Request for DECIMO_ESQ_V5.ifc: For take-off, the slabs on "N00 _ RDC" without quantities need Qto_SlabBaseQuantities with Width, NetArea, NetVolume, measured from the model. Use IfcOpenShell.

First a look at what the model holds.

```python
import ifcopenshell
import ifcopenshell.util.element
import ifcopenshell.util.unit

model = ifcopenshell.open("DECIMO_ESQ_V5.ifc")
print(model.schema)
for unit_type in ("LENGTHUNIT", "AREAUNIT", "VOLUMEUNIT"):
    print(unit_type, ifcopenshell.util.unit.calculate_unit_scale(model, unit_type))
storey = next(s for s in model.by_type("IfcBuildingStorey") if s.Name == "N00 _ RDC")
slabs = [e for e in ifcopenshell.util.element.get_decomposition(storey) if e.is_a("IfcSlab")]
for e in sorted(slabs, key=lambda e: e.id()):
    print(e.id(), e.is_a(), e.Name, list(ifcopenshell.util.element.get_psets(e, qtos_only=True)), sep=" | ")
```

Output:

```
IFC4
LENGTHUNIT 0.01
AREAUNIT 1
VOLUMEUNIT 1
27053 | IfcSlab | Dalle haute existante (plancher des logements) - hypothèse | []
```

```python
import ifcopenshell
import ifcopenshell.api.pset
import ifcopenshell.geom
import ifcopenshell.util.element
import ifcopenshell.util.shape
import ifcopenshell.util.unit

model = ifcopenshell.open("DECIMO_ESQ_V5.ifc")
unit_scale = ifcopenshell.util.unit.calculate_unit_scale(model)
area_scale = ifcopenshell.util.unit.calculate_unit_scale(model, "AREAUNIT")
volume_scale = ifcopenshell.util.unit.calculate_unit_scale(model, "VOLUMEUNIT")
settings = ifcopenshell.geom.settings()

storey = next(s for s in model.by_type("IfcBuildingStorey") if s.Name == "N00 _ RDC")
slabs = [e for e in ifcopenshell.util.element.get_decomposition(storey) if e.is_a("IfcSlab")]

for e in sorted(slabs, key=lambda e: e.id()):
    if ifcopenshell.util.element.get_psets(e, qtos_only=True, should_inherit=False):
        continue
    # Geometry comes back in metres, in the element's own axes.
    shape = ifcopenshell.geom.create_shape(settings, e)
    values = {
        "Width": ifcopenshell.util.shape.get_z(shape.geometry) / unit_scale,
        "NetArea": ifcopenshell.util.shape.get_footprint_area(shape.geometry) / area_scale,
        "NetVolume": ifcopenshell.util.shape.get_volume(shape.geometry) / volume_scale,
    }
    qto = ifcopenshell.api.pset.add_qto(model, product=e, name="Qto_SlabBaseQuantities")
    ifcopenshell.api.pset.edit_qto(model, qto=qto, properties=values)
    print(e.id(), {k: round(v, 3) for k, v in values.items()})

model.write("DECIMO_ESQ_V5-out.ifc")
```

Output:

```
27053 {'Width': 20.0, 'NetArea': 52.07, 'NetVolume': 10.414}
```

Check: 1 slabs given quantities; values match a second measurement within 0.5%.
